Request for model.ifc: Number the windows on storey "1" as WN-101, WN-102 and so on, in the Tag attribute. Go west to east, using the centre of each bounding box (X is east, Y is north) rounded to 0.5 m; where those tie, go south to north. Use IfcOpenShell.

First a look at what the model holds.

```python
import ifcopenshell
import ifcopenshell.util.element
import ifcopenshell.util.placement

model = ifcopenshell.open("model.ifc")
print(model.schema)
storey = next(s for s in model.by_type("IfcBuildingStorey") if s.Name == "1")
windows = [e for e in ifcopenshell.util.element.get_decomposition(storey) if e.is_a("IfcWindow")]
for e in sorted(windows, key=lambda e: e.id()):
    origin = ifcopenshell.util.placement.get_local_placement(e.ObjectPlacement)[:3, 3]
    print(e.id(), e.Tag, e.Name, origin.round(2) + 0.0, sep=" | ")
```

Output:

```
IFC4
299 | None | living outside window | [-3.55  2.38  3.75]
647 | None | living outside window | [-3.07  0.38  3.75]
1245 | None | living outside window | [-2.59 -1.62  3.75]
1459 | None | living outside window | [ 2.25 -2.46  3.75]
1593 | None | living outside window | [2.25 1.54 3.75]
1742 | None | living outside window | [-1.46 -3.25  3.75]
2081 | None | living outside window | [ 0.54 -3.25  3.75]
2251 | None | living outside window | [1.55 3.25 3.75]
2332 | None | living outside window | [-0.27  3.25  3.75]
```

```python
import ifcopenshell
import ifcopenshell.geom
import ifcopenshell.util.element
import ifcopenshell.util.shape

model = ifcopenshell.open("model.ifc")
settings = ifcopenshell.geom.settings()
settings.set("use-world-coords", True)


def centre(element):
    shape = ifcopenshell.geom.create_shape(settings, element)
    return ifcopenshell.util.shape.get_bbox_centroid(shape.geometry)


storey = next(s for s in model.by_type("IfcBuildingStorey") if s.Name == "1")
windows = [e for e in ifcopenshell.util.element.get_decomposition(storey) if e.is_a("IfcWindow")]

# Insertion points can sit at a corner or the storey origin, so sort by the geometry (in metres).
centres = {e: centre(e) for e in windows}
windows.sort(key=lambda e: (round(centres[e][0] / 0.5), centres[e][1]))

for i, e in enumerate(windows, start=1):
    number = f"WN-1{i:02d}"
    e.Tag = number
    print(e.id(), number)

model.write("model_updated.ifc")
```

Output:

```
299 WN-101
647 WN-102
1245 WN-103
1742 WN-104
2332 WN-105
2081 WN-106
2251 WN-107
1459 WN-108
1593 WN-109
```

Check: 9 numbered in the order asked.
